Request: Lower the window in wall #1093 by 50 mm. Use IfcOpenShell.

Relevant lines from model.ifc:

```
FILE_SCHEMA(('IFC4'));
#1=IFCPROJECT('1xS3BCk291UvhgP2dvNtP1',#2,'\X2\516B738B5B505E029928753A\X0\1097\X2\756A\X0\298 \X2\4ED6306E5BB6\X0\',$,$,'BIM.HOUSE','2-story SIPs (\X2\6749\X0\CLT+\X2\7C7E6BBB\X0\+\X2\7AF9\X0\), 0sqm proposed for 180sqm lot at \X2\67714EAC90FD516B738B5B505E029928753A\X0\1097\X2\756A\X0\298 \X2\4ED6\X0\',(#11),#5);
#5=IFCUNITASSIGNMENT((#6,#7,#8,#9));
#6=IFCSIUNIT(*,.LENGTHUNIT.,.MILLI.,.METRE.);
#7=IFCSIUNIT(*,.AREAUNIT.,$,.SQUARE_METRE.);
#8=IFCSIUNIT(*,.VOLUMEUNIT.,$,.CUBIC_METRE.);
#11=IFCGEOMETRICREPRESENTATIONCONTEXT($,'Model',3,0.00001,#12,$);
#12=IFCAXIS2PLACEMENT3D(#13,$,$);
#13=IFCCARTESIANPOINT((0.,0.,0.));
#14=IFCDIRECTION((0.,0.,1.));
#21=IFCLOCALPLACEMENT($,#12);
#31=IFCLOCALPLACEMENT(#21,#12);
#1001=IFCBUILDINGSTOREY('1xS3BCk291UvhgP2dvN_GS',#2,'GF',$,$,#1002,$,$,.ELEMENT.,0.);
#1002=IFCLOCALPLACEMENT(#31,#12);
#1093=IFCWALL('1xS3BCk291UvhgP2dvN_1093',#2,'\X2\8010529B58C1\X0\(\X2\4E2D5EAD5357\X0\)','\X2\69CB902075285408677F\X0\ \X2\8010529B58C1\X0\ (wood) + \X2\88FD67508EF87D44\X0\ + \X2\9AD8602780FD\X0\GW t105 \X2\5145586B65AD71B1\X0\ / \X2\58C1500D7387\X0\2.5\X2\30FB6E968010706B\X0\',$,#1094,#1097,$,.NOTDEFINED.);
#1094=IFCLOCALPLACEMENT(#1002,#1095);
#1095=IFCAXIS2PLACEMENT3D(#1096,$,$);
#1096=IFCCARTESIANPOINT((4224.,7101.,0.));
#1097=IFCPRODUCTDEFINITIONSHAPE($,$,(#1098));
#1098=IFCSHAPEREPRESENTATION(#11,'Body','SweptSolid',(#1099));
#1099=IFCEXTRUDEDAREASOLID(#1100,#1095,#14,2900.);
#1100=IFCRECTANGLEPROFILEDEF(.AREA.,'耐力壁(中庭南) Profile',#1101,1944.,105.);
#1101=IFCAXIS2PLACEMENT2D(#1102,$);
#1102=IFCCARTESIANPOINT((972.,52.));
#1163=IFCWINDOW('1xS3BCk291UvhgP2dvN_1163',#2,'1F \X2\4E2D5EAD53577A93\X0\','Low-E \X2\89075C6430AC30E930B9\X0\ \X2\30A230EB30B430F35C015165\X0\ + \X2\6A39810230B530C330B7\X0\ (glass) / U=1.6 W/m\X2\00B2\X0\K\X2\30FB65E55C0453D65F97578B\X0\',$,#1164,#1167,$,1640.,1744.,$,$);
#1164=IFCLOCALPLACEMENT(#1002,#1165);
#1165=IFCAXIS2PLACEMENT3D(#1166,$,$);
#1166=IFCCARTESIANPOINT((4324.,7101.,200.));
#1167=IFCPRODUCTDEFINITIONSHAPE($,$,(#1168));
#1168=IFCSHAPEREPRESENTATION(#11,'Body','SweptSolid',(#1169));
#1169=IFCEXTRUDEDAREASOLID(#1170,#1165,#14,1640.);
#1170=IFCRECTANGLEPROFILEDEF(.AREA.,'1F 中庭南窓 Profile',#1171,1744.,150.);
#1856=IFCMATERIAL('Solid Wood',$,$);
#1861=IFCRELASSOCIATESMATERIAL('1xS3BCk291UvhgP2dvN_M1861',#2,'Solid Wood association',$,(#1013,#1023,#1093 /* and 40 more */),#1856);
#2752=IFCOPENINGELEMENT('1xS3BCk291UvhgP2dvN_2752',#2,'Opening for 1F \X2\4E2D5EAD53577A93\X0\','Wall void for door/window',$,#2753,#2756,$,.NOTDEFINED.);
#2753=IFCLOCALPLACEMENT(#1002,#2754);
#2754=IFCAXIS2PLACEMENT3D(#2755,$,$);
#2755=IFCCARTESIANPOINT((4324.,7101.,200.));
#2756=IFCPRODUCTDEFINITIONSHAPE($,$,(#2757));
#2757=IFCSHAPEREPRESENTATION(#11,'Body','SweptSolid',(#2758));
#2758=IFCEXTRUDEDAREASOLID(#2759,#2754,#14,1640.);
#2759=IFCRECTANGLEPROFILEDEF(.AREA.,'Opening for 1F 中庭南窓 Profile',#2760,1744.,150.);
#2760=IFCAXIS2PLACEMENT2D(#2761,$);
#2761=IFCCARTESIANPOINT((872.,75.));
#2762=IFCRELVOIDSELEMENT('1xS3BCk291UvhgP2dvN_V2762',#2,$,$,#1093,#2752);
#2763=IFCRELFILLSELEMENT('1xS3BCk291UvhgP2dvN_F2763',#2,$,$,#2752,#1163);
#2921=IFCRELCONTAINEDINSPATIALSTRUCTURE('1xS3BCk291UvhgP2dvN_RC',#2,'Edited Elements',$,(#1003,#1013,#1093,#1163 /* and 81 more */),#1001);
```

```python
import numpy as np
import ifcopenshell
import ifcopenshell.api.geometry
import ifcopenshell.util.placement
import ifcopenshell.util.unit

model = ifcopenshell.open("model.ifc")
unit_scale = ifcopenshell.util.unit.calculate_unit_scale(model)

window = model.by_guid("1xS3BCk291UvhgP2dvN_1163")
opening = window.FillsVoids[0].RelatingOpeningElement
dz = -50.0

shift = np.array([0.0, 0.0, dz])
# The window is not placed relative to its opening, so move both.
for product in (opening, window):
    matrix = ifcopenshell.util.placement.get_local_placement(product.ObjectPlacement)
    matrix[:3, 3] += shift
    ifcopenshell.api.geometry.edit_object_placement(model, product=product, matrix=matrix, is_si=False)

print(f"moved by {dz * unit_scale:+.3f} m")

model.write("model_v2.ifc")
```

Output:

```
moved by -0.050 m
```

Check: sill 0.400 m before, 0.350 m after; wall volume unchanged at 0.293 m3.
